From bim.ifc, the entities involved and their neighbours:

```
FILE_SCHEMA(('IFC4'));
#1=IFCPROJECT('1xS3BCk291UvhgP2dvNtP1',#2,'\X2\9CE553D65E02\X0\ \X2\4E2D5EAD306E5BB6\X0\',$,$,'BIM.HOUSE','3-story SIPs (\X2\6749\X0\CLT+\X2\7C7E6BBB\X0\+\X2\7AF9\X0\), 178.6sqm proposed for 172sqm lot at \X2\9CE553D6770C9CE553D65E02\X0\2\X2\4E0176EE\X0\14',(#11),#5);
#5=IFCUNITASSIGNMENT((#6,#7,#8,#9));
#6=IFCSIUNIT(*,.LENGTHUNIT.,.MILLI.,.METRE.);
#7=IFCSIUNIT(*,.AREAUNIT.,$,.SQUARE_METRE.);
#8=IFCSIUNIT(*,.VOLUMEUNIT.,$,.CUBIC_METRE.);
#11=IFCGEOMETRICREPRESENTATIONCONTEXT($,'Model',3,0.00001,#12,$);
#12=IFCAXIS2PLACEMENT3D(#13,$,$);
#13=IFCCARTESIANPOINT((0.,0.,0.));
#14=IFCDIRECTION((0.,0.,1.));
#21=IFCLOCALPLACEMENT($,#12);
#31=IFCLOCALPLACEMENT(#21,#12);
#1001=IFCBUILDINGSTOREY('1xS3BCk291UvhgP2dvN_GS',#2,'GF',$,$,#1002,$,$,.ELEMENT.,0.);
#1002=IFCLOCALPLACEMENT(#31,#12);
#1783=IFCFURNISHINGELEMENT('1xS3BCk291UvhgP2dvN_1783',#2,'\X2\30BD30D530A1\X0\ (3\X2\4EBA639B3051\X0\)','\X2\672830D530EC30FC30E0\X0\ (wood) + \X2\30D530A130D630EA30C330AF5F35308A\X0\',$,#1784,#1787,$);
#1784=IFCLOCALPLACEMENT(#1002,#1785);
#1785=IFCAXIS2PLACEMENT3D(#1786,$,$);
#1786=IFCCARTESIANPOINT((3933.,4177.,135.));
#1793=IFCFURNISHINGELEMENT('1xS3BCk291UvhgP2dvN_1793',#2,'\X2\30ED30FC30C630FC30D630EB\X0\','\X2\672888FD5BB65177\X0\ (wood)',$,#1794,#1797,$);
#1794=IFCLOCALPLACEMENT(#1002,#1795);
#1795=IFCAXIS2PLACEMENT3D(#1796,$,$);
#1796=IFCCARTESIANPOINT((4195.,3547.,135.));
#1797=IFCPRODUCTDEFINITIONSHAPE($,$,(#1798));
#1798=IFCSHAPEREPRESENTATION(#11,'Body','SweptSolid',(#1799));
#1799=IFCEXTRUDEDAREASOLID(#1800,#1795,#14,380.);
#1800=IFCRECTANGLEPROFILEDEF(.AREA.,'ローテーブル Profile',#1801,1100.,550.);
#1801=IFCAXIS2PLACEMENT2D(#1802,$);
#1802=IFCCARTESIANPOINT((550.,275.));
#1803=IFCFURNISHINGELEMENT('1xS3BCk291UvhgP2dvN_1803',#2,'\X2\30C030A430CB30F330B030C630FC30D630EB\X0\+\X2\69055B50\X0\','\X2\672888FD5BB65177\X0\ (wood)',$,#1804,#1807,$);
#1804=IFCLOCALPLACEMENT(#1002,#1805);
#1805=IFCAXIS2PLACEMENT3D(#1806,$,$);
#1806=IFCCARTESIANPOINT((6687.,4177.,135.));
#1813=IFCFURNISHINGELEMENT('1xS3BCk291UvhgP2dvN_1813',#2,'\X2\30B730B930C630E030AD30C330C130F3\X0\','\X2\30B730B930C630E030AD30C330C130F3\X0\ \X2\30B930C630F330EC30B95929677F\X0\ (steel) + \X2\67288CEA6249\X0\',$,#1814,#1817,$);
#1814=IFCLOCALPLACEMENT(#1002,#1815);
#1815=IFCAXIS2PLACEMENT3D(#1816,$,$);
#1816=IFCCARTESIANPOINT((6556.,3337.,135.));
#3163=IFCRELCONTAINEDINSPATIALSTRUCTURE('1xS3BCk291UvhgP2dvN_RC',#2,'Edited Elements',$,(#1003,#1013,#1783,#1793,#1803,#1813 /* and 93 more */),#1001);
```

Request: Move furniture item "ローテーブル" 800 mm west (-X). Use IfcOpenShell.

```python
import ifcopenshell
import ifcopenshell.api.geometry
import ifcopenshell.util.placement

model = ifcopenshell.open("bim.ifc")

item = model.by_guid("1xS3BCk291UvhgP2dvN_1793")
matrix = ifcopenshell.util.placement.get_local_placement(item.ObjectPlacement)
matrix[0, 3] -= 800.0
ifcopenshell.api.geometry.edit_object_placement(model, product=item, matrix=matrix, is_si=False)

print(ifcopenshell.util.placement.get_local_placement(item.ObjectPlacement).round(3) + 0.0)

model.write("bim_updated.ifc")
```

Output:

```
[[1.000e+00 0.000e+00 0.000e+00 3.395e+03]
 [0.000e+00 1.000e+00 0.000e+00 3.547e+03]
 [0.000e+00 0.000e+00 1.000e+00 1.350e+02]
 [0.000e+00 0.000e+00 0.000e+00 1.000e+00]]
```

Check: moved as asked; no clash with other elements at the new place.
